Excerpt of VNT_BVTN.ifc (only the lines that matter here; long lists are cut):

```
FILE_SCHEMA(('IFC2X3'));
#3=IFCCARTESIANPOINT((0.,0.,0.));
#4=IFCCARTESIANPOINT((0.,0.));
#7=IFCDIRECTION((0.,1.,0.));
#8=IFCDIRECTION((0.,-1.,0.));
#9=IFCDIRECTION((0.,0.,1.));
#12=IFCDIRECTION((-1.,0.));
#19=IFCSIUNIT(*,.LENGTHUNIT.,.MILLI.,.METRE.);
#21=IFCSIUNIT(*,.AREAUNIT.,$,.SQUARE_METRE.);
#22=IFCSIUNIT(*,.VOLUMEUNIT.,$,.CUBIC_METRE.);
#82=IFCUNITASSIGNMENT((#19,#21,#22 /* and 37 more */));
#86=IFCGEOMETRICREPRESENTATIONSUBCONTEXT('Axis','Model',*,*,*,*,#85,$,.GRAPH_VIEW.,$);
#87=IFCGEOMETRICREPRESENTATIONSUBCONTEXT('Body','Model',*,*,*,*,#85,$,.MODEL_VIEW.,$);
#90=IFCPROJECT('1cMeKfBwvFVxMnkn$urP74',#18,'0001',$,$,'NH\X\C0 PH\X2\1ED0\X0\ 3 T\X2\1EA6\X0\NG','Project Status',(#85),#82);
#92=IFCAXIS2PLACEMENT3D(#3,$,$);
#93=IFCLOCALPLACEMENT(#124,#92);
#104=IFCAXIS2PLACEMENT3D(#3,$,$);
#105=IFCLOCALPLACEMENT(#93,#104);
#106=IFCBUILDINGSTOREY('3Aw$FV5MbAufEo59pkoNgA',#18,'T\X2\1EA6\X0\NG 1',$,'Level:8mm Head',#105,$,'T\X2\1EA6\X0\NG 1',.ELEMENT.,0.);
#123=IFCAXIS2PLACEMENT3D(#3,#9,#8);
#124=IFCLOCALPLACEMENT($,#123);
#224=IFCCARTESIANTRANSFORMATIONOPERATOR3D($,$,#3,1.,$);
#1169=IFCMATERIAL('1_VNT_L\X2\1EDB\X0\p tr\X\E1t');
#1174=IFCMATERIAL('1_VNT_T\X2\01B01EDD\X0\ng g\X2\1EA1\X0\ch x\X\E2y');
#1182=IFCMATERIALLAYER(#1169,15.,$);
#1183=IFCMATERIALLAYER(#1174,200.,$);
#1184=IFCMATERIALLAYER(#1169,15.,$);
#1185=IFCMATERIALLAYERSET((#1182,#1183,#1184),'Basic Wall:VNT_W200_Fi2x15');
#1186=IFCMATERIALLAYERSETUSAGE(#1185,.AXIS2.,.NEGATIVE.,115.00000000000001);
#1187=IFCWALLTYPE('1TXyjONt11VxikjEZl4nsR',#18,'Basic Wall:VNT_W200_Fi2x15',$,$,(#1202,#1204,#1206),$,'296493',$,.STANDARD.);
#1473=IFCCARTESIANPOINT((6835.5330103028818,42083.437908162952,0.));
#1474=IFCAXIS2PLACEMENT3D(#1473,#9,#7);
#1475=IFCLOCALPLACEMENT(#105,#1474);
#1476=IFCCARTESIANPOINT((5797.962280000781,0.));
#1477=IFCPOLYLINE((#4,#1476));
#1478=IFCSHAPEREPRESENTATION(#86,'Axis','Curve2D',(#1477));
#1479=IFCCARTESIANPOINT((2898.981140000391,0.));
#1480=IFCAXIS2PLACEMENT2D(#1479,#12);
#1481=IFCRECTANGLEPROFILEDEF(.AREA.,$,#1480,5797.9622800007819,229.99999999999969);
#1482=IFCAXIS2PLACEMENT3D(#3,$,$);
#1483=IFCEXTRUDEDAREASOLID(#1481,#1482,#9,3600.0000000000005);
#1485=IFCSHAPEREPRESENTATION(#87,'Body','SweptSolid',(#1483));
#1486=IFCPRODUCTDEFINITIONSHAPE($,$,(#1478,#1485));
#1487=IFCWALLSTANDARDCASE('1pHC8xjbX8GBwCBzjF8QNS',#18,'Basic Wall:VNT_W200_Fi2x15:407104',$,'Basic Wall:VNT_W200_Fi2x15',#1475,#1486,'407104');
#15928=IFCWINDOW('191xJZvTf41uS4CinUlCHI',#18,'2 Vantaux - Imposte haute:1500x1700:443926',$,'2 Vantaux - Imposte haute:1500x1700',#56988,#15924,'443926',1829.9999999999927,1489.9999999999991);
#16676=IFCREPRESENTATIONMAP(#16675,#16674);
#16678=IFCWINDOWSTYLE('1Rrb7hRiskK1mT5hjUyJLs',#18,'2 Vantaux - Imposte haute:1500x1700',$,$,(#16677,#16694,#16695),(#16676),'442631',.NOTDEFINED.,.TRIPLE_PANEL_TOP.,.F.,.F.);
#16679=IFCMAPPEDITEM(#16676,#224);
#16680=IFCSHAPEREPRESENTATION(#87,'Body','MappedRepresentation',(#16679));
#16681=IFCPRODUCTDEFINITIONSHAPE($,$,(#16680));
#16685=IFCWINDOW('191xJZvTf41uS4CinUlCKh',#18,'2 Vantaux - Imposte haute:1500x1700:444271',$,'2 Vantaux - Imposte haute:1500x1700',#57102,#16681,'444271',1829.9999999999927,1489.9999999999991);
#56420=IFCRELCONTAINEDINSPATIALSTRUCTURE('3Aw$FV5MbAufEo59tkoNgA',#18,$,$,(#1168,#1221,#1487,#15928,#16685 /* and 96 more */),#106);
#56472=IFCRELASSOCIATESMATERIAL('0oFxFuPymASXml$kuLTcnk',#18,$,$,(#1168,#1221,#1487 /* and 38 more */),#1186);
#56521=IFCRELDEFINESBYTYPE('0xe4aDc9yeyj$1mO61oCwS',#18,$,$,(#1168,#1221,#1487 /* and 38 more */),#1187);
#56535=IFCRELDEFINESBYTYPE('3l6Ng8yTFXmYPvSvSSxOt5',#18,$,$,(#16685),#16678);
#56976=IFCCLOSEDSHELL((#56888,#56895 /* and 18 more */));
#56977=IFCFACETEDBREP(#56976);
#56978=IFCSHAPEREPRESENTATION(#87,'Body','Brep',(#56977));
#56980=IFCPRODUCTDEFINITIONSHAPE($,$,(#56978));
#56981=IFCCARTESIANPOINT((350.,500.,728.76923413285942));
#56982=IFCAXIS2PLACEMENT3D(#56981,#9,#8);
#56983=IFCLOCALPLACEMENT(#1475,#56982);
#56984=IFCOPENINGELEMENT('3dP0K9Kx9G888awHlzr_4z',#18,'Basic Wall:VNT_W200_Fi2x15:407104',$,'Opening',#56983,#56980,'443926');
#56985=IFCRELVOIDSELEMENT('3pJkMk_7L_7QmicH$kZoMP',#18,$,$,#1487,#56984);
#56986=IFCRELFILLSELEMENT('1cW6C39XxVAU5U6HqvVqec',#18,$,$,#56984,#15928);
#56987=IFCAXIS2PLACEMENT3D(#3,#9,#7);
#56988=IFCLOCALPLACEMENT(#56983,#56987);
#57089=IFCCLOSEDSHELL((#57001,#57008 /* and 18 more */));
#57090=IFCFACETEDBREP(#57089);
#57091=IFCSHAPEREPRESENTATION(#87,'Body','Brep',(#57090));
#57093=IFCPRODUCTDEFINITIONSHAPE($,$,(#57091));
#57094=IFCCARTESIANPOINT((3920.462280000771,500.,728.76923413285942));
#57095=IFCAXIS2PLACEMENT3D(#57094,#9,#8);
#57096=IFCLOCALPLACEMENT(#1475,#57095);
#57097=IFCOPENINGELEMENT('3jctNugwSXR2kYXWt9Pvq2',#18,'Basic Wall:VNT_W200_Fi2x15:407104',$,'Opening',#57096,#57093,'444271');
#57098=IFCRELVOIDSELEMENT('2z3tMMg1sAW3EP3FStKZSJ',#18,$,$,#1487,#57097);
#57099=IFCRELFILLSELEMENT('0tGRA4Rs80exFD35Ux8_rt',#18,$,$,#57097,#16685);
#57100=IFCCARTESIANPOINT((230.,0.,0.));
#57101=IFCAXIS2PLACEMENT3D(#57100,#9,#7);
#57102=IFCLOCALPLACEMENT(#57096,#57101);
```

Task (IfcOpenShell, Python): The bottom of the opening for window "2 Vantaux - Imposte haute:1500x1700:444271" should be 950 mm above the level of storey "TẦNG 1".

```python
import numpy as np
import ifcopenshell
import ifcopenshell.api.geometry
import ifcopenshell.geom
import ifcopenshell.util.element
import ifcopenshell.util.placement
import ifcopenshell.util.shape
import ifcopenshell.util.unit

model = ifcopenshell.open("VNT_BVTN.ifc")
unit_scale = ifcopenshell.util.unit.calculate_unit_scale(model)

window = model.by_guid("191xJZvTf41uS4CinUlCKh")
opening = window.FillsVoids[0].RelatingOpeningElement
storey = ifcopenshell.util.element.get_container(window, ifc_class="IfcBuildingStorey")
level = ifcopenshell.util.placement.get_local_placement(storey.ObjectPlacement)[2, 3]

# The opening's origin need not be at the sill, so measure its lowest point.
shape = ifcopenshell.geom.create_shape(ifcopenshell.geom.settings(), opening)
bottom = ifcopenshell.util.shape.get_shape_bottom_elevation(shape, shape.geometry) / unit_scale
dz = level + 0.95 / unit_scale - bottom

shift = np.array([0.0, 0.0, dz])
# The window is placed relative to its opening, so it follows when the opening moves.
matrix = ifcopenshell.util.placement.get_local_placement(opening.ObjectPlacement)
matrix[:3, 3] += shift
ifcopenshell.api.geometry.edit_object_placement(
    model, product=opening, matrix=matrix, is_si=False, should_transform_children=True
)

print(f"moved by {dz * unit_scale:+.3f} m")

model.write("VNT_BVTN_edited.ifc")
```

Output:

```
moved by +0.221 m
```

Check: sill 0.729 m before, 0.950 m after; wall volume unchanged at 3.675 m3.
